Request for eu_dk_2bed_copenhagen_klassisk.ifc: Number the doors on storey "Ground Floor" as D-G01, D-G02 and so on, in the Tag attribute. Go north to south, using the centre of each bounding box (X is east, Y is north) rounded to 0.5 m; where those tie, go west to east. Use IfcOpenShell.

First a look at what the model holds.

```python
import ifcopenshell
import ifcopenshell.util.element
import ifcopenshell.util.placement

model = ifcopenshell.open("eu_dk_2bed_copenhagen_klassisk.ifc")
print(model.schema)
storey = next(s for s in model.by_type("IfcBuildingStorey") if s.Name == "Ground Floor")
doors = [e for e in ifcopenshell.util.element.get_decomposition(storey) if e.is_a("IfcDoor")]
for e in sorted(doors, key=lambda e: e.id()):
    origin = ifcopenshell.util.placement.get_local_placement(e.ObjectPlacement)[:3, 3]
    print(e.id(), e.Tag, e.Name, origin.round(2) + 0.0, sep=" | ")
```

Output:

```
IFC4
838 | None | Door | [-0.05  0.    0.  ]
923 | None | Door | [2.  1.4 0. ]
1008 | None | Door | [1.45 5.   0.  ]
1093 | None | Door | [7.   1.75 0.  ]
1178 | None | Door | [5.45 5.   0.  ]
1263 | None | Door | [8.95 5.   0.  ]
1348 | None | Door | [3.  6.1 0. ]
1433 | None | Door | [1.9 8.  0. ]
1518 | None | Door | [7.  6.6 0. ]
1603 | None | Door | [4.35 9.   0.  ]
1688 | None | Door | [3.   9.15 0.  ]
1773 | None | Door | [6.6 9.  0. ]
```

```python
import ifcopenshell
import ifcopenshell.geom
import ifcopenshell.util.element
import ifcopenshell.util.shape

model = ifcopenshell.open("eu_dk_2bed_copenhagen_klassisk.ifc")
settings = ifcopenshell.geom.settings()
settings.set("use-world-coords", True)


def centre(element):
    shape = ifcopenshell.geom.create_shape(settings, element)
    return ifcopenshell.util.shape.get_bbox_centroid(shape.geometry)


storey = next(s for s in model.by_type("IfcBuildingStorey") if s.Name == "Ground Floor")
doors = [e for e in ifcopenshell.util.element.get_decomposition(storey) if e.is_a("IfcDoor")]

# Insertion points can sit at a corner or the storey origin, so sort by the geometry (in metres).
centres = {e: centre(e) for e in doors}
doors.sort(key=lambda e: (-round(centres[e][1] / 0.5), centres[e][0]))

for i, e in enumerate(doors, start=1):
    number = f"D-G{i:02d}"
    e.Tag = number
    print(e.id(), number)

model.write("eu_dk_2bed_copenhagen_klassisk_updated.ifc")
```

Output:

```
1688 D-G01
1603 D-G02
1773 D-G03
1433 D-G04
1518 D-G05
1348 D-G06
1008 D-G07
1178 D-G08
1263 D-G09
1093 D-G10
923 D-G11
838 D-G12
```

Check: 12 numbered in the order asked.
